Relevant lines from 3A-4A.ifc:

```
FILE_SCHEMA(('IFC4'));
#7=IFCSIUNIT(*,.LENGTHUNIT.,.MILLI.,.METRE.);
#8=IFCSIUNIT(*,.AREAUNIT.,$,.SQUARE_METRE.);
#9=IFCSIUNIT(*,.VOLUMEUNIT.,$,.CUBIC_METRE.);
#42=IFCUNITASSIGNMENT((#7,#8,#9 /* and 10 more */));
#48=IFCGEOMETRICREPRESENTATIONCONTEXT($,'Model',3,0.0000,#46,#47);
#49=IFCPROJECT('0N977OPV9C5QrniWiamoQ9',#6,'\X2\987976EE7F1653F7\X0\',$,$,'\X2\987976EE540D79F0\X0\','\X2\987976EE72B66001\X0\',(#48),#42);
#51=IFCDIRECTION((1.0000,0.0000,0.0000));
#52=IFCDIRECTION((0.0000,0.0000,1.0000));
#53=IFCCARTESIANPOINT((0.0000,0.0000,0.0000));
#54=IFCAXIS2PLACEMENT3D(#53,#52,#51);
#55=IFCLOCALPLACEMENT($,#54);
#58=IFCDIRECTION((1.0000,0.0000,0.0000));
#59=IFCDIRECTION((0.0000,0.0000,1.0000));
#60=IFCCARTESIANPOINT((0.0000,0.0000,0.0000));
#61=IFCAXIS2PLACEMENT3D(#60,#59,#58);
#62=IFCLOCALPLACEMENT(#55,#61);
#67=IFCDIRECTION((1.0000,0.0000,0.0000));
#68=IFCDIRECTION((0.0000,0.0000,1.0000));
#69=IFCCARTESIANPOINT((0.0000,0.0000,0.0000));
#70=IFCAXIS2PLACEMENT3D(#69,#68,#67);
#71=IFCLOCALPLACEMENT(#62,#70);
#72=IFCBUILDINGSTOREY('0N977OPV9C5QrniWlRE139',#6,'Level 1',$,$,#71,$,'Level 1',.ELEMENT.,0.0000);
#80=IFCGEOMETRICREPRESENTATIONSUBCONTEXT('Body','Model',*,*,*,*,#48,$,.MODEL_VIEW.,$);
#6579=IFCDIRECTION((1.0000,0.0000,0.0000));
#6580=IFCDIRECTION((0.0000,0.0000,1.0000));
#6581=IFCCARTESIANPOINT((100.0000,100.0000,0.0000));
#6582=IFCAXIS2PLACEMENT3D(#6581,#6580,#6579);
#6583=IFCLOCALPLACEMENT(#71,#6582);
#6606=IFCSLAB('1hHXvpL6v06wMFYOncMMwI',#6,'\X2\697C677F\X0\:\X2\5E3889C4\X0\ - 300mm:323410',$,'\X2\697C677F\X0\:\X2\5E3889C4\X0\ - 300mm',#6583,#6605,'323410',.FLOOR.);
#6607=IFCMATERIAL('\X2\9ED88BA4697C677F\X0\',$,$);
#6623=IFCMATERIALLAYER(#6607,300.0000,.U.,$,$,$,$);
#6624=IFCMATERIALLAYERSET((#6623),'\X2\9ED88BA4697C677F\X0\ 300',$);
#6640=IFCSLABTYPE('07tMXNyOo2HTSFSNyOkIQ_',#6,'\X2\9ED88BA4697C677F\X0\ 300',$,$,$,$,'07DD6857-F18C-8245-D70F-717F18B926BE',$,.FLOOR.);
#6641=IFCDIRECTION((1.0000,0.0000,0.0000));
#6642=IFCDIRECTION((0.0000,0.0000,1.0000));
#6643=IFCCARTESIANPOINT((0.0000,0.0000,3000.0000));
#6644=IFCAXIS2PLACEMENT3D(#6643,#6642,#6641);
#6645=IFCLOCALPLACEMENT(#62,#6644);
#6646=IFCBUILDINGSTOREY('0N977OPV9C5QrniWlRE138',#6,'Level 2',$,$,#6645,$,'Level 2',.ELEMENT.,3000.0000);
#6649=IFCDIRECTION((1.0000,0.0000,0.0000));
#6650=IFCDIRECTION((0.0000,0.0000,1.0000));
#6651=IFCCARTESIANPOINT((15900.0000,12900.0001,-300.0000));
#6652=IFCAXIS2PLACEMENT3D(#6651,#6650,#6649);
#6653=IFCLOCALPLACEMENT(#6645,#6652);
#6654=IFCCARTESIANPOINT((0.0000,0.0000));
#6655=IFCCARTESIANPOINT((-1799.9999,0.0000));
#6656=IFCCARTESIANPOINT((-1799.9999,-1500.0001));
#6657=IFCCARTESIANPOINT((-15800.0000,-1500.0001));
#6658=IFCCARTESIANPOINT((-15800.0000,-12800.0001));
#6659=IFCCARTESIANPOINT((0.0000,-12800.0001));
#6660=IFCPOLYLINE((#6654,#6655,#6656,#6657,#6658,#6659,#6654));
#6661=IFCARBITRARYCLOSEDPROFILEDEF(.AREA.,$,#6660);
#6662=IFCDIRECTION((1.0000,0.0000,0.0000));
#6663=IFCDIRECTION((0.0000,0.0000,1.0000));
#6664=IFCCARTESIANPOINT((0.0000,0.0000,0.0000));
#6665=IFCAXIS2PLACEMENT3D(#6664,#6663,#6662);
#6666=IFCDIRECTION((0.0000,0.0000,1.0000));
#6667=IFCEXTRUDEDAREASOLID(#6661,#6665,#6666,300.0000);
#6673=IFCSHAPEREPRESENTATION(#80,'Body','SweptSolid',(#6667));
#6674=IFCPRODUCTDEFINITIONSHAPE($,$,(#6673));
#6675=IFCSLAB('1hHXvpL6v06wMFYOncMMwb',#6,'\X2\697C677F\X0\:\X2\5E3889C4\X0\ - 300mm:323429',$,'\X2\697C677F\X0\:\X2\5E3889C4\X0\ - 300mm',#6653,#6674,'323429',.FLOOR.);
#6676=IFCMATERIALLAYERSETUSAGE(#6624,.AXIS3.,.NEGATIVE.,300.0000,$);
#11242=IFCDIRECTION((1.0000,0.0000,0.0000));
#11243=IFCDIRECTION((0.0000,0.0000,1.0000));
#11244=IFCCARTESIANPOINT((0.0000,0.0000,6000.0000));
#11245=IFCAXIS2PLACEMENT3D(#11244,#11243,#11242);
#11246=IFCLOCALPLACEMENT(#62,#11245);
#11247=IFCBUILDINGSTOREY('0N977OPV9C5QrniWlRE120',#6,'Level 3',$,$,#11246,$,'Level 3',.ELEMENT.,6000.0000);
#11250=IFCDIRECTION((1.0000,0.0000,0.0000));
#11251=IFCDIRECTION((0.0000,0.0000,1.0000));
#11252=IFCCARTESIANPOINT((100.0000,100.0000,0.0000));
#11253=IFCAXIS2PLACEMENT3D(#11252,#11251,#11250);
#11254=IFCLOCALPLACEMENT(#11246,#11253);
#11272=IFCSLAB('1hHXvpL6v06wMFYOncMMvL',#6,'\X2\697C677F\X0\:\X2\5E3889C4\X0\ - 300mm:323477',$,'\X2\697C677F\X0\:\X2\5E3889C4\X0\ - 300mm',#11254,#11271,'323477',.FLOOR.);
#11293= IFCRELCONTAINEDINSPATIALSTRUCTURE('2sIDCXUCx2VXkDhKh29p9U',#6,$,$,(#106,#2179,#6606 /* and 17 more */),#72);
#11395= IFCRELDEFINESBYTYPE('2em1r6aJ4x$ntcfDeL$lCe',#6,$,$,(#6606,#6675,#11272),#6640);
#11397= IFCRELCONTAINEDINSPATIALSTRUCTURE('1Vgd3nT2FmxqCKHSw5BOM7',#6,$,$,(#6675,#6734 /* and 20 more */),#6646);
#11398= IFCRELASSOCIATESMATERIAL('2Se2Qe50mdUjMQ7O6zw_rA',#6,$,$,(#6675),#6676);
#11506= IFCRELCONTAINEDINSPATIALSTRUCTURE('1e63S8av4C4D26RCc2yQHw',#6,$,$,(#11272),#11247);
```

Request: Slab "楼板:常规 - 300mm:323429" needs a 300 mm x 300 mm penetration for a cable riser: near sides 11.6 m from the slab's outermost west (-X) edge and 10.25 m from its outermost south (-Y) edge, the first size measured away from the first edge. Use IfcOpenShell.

```python
import numpy as np
import ifcopenshell
import ifcopenshell.api.feature
import ifcopenshell.api.geometry
import ifcopenshell.api.root
import ifcopenshell.geom
import ifcopenshell.util.placement
import ifcopenshell.util.representation
import ifcopenshell.util.shape
import ifcopenshell.util.unit

model = ifcopenshell.open("3A-4A.ifc")
unit_scale = ifcopenshell.util.unit.calculate_unit_scale(model)
settings = ifcopenshell.geom.settings()


def volume(element):
    """Net volume in cubic metres, openings subtracted."""
    shape = ifcopenshell.geom.create_shape(settings, element)
    return ifcopenshell.util.shape.get_volume(shape.geometry)


slab = model.by_id(6675)
before = volume(slab)

# Extent in the slab's own axes, in metres. The edges named are its -X and -Y sides.
slab_shape = ifcopenshell.geom.create_shape(settings, slab)
vertices = ifcopenshell.util.shape.get_vertices(slab_shape.geometry)
x_min, y_min, bottom = vertices.min(axis=0)
top = vertices[:, 2].max()

opening = ifcopenshell.api.root.create_entity(model, ifc_class="IfcOpeningElement", name="Cable riser opening", predefined_type="OPENING")
context = ifcopenshell.util.representation.get_context(model, "Model", "Body", "MODEL_VIEW")
width, depth = 0.3, 0.3
outline = [(0.0, 0.0), (width, 0.0), (width, depth), (0.0, depth), (0.0, 0.0)]
# Overshoot both faces by 50 mm so the cut is clean.
shape = ifcopenshell.api.geometry.add_slab_representation(
    model, context=context, depth=top - bottom + 0.1, polyline=outline
)
ifcopenshell.api.geometry.assign_representation(model, product=opening, representation=shape)

matrix = ifcopenshell.util.placement.get_local_placement(slab.ObjectPlacement)
matrix[:, 3] = matrix @ np.append(np.array([x_min + 11.6, y_min + 10.25, bottom - 0.05]) / unit_scale, 1.0)
ifcopenshell.api.geometry.edit_object_placement(model, product=opening, matrix=matrix, is_si=False)
ifcopenshell.api.feature.add_feature(model, feature=opening, element=slab)

after = volume(slab)

print(f"slab volume {before:.3f} -> {after:.3f} m3")

model.write("3A-4A_edited.ifc")
```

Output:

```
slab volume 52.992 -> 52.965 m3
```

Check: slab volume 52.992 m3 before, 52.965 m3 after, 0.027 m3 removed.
